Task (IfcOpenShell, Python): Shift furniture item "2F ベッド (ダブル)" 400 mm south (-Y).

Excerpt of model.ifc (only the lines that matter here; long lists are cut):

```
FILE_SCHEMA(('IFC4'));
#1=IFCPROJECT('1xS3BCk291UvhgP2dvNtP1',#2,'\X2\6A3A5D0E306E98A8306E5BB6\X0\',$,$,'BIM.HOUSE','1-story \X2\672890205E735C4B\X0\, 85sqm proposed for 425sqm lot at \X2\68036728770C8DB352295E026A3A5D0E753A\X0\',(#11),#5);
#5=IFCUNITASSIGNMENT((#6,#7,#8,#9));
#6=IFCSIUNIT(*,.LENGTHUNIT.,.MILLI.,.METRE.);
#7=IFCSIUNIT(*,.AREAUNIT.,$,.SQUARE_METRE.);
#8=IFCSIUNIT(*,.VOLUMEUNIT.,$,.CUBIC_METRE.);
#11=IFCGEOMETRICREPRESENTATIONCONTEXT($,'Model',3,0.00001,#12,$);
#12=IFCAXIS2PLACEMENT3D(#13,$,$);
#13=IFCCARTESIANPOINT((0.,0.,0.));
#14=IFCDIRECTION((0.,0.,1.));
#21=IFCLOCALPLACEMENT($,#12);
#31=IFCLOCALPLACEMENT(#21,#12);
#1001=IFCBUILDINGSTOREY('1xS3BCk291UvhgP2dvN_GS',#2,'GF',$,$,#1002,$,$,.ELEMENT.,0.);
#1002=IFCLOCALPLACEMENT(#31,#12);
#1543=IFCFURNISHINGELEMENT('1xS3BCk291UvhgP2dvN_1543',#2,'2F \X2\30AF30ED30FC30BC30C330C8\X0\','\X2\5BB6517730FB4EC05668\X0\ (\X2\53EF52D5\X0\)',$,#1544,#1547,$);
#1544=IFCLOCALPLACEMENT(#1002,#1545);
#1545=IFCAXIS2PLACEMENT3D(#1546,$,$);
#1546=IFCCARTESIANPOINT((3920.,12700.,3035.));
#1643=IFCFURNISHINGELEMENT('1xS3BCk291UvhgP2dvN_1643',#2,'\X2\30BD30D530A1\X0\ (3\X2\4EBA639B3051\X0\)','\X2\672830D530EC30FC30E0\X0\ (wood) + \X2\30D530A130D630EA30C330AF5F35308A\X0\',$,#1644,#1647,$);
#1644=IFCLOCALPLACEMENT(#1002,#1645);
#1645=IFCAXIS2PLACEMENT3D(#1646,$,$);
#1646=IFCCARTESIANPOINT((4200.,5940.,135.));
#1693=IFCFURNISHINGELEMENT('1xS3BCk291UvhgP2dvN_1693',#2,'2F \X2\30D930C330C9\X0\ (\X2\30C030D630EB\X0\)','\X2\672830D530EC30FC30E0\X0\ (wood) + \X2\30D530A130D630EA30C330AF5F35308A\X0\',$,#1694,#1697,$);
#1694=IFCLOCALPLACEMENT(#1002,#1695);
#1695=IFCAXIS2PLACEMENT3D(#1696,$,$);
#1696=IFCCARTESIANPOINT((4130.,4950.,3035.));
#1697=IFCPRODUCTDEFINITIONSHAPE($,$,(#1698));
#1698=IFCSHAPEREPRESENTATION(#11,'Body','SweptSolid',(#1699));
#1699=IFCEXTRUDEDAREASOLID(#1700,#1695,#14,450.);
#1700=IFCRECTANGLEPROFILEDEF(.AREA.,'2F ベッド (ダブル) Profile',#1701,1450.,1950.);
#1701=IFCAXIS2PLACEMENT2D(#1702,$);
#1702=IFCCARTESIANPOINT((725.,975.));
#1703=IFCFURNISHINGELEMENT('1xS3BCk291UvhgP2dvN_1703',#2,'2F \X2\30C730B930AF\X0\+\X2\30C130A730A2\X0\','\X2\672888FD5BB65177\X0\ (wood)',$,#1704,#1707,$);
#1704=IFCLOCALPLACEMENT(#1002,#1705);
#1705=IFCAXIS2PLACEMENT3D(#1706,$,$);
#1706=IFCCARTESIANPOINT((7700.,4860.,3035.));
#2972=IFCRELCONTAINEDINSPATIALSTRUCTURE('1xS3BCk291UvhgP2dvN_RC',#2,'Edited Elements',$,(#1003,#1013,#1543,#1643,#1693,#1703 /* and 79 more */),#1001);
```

```python
import ifcopenshell
import ifcopenshell.api.geometry
import ifcopenshell.util.placement
import ifcopenshell.util.unit

model = ifcopenshell.open("model.ifc")
unit_scale = ifcopenshell.util.unit.calculate_unit_scale(model)

item = model.by_id(1693)
matrix = ifcopenshell.util.placement.get_local_placement(item.ObjectPlacement)
matrix[1, 3] -= 0.4 / unit_scale
ifcopenshell.api.geometry.edit_object_placement(model, product=item, matrix=matrix, is_si=False)

print(ifcopenshell.util.placement.get_local_placement(item.ObjectPlacement).round(3) + 0.0)

model.write("model_updated.ifc")
```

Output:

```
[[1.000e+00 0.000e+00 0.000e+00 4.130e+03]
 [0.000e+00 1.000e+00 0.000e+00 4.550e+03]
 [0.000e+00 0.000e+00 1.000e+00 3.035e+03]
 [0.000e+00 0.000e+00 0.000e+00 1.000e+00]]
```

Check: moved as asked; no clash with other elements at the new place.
